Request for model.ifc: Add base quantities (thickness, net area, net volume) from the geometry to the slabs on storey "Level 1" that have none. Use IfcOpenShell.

First a look at what the model holds.

```python
import ifcopenshell
import ifcopenshell.util.element
import ifcopenshell.util.unit

model = ifcopenshell.open("model.ifc")
print(model.schema)
for unit_type in ("LENGTHUNIT", "AREAUNIT", "VOLUMEUNIT"):
    print(unit_type, ifcopenshell.util.unit.calculate_unit_scale(model, unit_type))
storey = next(s for s in model.by_type("IfcBuildingStorey") if s.Name == "Level 1")
slabs = [e for e in ifcopenshell.util.element.get_decomposition(storey) if e.is_a("IfcSlab")]
for e in sorted(slabs, key=lambda e: e.id()):
    print(e.id(), e.is_a(), e.Name, list(ifcopenshell.util.element.get_psets(e, qtos_only=True)), sep=" | ")
```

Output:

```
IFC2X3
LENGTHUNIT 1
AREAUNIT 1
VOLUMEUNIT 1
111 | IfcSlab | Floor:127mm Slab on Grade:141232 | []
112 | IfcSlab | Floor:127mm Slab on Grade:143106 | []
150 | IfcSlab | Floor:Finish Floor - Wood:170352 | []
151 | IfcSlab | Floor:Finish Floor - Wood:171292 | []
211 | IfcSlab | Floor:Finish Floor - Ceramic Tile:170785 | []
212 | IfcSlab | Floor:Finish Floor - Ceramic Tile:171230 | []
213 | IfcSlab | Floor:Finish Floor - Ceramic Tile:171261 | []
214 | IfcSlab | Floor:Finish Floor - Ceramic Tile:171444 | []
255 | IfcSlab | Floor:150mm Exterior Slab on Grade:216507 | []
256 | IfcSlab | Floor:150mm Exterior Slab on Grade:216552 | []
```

```python
import ifcopenshell
import ifcopenshell.api.pset
import ifcopenshell.geom
import ifcopenshell.util.element
import ifcopenshell.util.shape
import ifcopenshell.util.unit

model = ifcopenshell.open("model.ifc")
unit_scale = ifcopenshell.util.unit.calculate_unit_scale(model)
area_scale = ifcopenshell.util.unit.calculate_unit_scale(model, "AREAUNIT")
volume_scale = ifcopenshell.util.unit.calculate_unit_scale(model, "VOLUMEUNIT")
settings = ifcopenshell.geom.settings()

storey = next(s for s in model.by_type("IfcBuildingStorey") if s.Name == "Level 1")
slabs = [e for e in ifcopenshell.util.element.get_decomposition(storey) if e.is_a("IfcSlab")]

for e in sorted(slabs, key=lambda e: e.id()):
    if ifcopenshell.util.element.get_psets(e, qtos_only=True, should_inherit=False):
        continue
    # Geometry comes back in metres, in the element's own axes.
    shape = ifcopenshell.geom.create_shape(settings, e)
    values = {
        "Width": ifcopenshell.util.shape.get_z(shape.geometry) / unit_scale,
        "NetArea": ifcopenshell.util.shape.get_footprint_area(shape.geometry) / area_scale,
        "NetVolume": ifcopenshell.util.shape.get_volume(shape.geometry) / volume_scale,
    }
    qto = ifcopenshell.api.pset.add_qto(model, product=e, name="BaseQuantities")
    ifcopenshell.api.pset.edit_qto(model, qto=qto, properties=values)
    print(e.id(), {k: round(v, 3) for k, v in values.items()})

model.write("model_rev.ifc")
```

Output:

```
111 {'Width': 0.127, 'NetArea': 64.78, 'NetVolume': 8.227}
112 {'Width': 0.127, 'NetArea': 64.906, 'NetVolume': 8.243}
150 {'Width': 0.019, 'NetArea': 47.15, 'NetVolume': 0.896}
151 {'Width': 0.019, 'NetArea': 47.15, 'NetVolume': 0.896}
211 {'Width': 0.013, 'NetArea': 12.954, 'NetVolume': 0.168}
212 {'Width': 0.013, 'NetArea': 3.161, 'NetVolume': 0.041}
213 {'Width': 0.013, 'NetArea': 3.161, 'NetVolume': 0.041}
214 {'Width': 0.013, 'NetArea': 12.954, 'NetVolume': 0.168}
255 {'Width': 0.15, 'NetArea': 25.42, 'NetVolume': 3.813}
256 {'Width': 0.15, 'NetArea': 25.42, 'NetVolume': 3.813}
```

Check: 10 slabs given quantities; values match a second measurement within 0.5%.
